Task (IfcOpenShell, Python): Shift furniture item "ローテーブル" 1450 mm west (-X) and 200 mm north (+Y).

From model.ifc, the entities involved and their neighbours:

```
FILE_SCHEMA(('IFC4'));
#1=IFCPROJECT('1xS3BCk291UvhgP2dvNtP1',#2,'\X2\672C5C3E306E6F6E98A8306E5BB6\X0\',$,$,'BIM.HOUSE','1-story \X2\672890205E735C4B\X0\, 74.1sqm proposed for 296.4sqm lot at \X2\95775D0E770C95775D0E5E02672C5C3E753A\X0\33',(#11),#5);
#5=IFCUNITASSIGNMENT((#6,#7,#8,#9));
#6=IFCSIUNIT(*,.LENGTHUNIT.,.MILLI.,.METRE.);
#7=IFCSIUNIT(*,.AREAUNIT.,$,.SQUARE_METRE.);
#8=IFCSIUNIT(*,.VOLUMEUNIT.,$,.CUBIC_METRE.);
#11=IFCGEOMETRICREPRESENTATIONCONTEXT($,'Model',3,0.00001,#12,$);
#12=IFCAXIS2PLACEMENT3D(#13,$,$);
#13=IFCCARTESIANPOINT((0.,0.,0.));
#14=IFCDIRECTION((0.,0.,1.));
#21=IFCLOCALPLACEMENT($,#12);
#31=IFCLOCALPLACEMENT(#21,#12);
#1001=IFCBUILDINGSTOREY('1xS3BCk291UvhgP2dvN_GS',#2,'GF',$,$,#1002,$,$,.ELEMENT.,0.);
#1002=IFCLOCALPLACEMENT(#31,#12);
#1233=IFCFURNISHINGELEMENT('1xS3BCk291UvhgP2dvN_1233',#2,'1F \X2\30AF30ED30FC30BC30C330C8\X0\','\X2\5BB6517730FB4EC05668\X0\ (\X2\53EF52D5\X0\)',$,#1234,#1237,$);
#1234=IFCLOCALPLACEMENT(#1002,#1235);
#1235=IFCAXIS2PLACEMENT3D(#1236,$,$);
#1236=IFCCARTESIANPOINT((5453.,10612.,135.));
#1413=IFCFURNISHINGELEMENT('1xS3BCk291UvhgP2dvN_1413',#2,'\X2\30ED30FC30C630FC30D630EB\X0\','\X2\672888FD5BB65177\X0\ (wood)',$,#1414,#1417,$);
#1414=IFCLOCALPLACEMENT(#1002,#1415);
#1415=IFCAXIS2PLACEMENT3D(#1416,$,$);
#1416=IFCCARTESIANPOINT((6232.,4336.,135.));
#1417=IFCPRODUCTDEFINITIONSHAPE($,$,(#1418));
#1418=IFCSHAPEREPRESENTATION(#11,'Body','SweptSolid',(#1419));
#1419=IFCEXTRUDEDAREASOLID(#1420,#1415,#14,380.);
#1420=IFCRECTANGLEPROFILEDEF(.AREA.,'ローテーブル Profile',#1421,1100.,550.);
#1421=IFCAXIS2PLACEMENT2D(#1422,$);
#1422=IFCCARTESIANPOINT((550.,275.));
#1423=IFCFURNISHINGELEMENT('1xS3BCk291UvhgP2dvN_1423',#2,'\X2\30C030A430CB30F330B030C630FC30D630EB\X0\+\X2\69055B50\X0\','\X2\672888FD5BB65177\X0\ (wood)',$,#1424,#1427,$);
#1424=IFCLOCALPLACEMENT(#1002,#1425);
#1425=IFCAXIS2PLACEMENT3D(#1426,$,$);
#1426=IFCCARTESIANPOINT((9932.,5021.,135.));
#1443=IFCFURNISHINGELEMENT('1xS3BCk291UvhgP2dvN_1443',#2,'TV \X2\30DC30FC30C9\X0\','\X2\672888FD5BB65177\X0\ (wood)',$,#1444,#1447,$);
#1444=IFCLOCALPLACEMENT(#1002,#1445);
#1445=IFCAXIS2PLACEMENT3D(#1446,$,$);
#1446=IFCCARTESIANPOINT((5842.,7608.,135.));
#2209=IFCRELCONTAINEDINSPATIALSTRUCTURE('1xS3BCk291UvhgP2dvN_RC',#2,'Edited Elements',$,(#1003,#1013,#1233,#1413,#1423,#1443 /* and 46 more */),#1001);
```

```python
import ifcopenshell
import ifcopenshell.api.geometry
import ifcopenshell.util.placement

model = ifcopenshell.open("model.ifc")

item = model.by_guid("1xS3BCk291UvhgP2dvN_1413")
matrix = ifcopenshell.util.placement.get_local_placement(item.ObjectPlacement)
matrix[0, 3] -= 1450.0
matrix[1, 3] += 200.0
ifcopenshell.api.geometry.edit_object_placement(model, product=item, matrix=matrix, is_si=False)

print(ifcopenshell.util.placement.get_local_placement(item.ObjectPlacement).round(3) + 0.0)

model.write("model_rev.ifc")
```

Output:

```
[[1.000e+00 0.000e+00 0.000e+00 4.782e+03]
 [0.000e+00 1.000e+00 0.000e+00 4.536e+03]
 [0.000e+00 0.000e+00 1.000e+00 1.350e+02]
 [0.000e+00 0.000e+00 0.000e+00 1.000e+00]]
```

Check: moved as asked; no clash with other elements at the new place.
